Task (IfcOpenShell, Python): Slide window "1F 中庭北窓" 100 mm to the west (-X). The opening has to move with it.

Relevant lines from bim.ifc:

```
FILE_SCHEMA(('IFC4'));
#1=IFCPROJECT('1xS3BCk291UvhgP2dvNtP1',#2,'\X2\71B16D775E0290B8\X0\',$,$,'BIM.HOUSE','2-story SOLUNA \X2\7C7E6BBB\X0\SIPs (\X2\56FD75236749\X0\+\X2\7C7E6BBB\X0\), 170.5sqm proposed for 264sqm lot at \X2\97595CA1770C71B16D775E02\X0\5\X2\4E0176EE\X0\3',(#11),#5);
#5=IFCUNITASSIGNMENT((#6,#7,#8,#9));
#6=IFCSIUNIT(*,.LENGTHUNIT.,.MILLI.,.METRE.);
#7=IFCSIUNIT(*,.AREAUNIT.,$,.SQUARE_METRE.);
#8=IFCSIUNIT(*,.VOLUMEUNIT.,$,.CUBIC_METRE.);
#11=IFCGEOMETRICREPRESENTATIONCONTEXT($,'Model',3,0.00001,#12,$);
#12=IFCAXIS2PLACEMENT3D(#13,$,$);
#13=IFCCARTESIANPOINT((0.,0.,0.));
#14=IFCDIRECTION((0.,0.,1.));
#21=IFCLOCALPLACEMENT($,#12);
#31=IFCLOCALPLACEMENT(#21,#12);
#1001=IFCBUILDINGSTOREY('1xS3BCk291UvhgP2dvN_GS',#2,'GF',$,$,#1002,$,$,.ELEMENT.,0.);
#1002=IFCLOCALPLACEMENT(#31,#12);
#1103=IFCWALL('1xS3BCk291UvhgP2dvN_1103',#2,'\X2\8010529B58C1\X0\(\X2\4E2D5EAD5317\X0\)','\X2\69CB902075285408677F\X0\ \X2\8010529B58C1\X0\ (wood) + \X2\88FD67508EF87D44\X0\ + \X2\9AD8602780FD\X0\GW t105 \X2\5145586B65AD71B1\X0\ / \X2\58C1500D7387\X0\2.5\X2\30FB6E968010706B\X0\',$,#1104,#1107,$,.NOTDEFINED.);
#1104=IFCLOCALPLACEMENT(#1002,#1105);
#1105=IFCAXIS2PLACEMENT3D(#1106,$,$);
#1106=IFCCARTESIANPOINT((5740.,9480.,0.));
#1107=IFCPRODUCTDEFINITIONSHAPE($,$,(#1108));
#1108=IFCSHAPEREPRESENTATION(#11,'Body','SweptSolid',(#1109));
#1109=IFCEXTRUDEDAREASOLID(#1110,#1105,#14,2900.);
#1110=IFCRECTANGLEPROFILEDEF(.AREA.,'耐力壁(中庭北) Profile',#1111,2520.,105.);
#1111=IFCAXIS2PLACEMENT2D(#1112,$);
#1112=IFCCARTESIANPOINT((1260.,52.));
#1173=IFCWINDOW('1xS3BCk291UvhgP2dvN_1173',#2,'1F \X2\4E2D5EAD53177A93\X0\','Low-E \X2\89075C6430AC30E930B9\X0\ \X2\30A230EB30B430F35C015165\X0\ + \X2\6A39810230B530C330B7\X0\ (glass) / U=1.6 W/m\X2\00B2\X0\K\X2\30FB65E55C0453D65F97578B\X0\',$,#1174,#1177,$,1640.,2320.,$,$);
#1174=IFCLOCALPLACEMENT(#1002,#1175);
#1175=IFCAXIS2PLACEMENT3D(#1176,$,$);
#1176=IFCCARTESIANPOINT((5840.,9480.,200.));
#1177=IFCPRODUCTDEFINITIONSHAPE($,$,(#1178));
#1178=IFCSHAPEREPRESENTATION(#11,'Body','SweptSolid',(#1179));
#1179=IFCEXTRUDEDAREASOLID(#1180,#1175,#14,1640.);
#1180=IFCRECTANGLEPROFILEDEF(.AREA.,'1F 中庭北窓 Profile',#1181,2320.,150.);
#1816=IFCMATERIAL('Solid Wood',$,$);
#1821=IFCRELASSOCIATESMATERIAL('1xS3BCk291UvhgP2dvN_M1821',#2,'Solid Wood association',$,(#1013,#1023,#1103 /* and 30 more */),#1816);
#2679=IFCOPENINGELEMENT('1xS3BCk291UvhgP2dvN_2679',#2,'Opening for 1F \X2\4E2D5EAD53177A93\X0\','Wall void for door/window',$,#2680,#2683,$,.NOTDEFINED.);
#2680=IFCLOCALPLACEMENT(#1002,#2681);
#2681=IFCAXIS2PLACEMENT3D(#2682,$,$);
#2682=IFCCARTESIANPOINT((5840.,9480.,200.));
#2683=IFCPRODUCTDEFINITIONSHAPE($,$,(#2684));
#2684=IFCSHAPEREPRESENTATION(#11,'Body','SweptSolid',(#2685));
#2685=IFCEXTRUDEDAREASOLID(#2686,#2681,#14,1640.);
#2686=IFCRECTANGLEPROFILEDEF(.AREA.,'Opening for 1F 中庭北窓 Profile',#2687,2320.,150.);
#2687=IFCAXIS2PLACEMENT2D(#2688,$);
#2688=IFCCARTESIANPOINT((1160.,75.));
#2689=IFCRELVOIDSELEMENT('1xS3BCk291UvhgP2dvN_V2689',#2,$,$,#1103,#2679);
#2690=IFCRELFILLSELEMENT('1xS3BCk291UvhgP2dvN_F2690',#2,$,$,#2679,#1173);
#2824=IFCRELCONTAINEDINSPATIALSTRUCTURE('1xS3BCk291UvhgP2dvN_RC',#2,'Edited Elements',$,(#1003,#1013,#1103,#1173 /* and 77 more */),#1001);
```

```python
import ifcopenshell
import ifcopenshell.api.geometry
import ifcopenshell.util.placement
import ifcopenshell.util.unit

model = ifcopenshell.open("bim.ifc")
unit_scale = ifcopenshell.util.unit.calculate_unit_scale(model)

window = model.by_guid("1xS3BCk291UvhgP2dvN_1173")
opening = window.FillsVoids[0].RelatingOpeningElement
wall = opening.VoidsElements[0].RelatingBuildingElement

wall_matrix = ifcopenshell.util.placement.get_local_placement(wall.ObjectPlacement)
shift = wall_matrix[:3, 0] * -0.1 / unit_scale
before = ifcopenshell.util.placement.get_local_placement(window.ObjectPlacement)[:3, 3].copy()

# The window is not placed relative to its opening, so move both.
for product in (opening, window):
    matrix = ifcopenshell.util.placement.get_local_placement(product.ObjectPlacement)
    matrix[:3, 3] += shift
    ifcopenshell.api.geometry.edit_object_placement(model, product=product, matrix=matrix, is_si=False)

after = ifcopenshell.util.placement.get_local_placement(window.ObjectPlacement)[:3, 3]
print("window moved by", (after - before).round(3) + 0.0)

model.write("bim_edited.ifc")
```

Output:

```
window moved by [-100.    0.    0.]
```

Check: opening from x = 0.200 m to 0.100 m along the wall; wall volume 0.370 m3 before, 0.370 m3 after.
